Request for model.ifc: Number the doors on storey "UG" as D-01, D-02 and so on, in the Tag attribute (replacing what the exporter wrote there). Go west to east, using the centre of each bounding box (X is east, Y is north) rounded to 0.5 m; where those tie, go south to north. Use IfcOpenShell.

First a look at what the model holds.

```python
import ifcopenshell
import ifcopenshell.util.element
import ifcopenshell.util.placement

model = ifcopenshell.open("model.ifc")
print(model.schema)
storey = next(s for s in model.by_type("IfcBuildingStorey") if s.Name == "UG")
doors = [e for e in ifcopenshell.util.element.get_decomposition(storey) if e.is_a("IfcDoor")]
for e in sorted(doors, key=lambda e: e.id()):
    origin = ifcopenshell.util.placement.get_local_placement(e.ObjectPlacement)[:3, 3]
    print(e.id(), e.Tag, e.Name, origin.round(2) + 0.0, sep=" | ")
```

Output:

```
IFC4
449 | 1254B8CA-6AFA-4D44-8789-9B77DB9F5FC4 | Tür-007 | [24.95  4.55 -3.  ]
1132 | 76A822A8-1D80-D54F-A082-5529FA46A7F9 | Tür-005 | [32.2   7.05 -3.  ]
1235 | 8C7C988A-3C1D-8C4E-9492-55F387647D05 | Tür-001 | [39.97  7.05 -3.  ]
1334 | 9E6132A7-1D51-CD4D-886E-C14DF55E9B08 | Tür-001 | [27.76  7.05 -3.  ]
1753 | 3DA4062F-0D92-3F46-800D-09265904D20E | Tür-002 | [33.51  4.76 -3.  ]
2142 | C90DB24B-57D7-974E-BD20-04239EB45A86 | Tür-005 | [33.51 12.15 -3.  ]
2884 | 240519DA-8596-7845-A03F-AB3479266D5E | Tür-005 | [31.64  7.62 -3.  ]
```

```python
import ifcopenshell
import ifcopenshell.geom
import ifcopenshell.util.element
import ifcopenshell.util.shape

model = ifcopenshell.open("model.ifc")
settings = ifcopenshell.geom.settings()
settings.set("use-world-coords", True)


def centre(element):
    shape = ifcopenshell.geom.create_shape(settings, element)
    return ifcopenshell.util.shape.get_bbox_centroid(shape.geometry)


storey = next(s for s in model.by_type("IfcBuildingStorey") if s.Name == "UG")
doors = [e for e in ifcopenshell.util.element.get_decomposition(storey) if e.is_a("IfcDoor")]

# Insertion points can sit at a corner or the storey origin, so sort by the geometry (in metres).
centres = {e: centre(e) for e in doors}
doors.sort(key=lambda e: (round(centres[e][0] / 0.5), centres[e][1]))

for i, e in enumerate(doors, start=1):
    number = f"D-{i:02d}"
    e.Tag = number
    print(e.id(), number)

model.write("model-out.ifc")
```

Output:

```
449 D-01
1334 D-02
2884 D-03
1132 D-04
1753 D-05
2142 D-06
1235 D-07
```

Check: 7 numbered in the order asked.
